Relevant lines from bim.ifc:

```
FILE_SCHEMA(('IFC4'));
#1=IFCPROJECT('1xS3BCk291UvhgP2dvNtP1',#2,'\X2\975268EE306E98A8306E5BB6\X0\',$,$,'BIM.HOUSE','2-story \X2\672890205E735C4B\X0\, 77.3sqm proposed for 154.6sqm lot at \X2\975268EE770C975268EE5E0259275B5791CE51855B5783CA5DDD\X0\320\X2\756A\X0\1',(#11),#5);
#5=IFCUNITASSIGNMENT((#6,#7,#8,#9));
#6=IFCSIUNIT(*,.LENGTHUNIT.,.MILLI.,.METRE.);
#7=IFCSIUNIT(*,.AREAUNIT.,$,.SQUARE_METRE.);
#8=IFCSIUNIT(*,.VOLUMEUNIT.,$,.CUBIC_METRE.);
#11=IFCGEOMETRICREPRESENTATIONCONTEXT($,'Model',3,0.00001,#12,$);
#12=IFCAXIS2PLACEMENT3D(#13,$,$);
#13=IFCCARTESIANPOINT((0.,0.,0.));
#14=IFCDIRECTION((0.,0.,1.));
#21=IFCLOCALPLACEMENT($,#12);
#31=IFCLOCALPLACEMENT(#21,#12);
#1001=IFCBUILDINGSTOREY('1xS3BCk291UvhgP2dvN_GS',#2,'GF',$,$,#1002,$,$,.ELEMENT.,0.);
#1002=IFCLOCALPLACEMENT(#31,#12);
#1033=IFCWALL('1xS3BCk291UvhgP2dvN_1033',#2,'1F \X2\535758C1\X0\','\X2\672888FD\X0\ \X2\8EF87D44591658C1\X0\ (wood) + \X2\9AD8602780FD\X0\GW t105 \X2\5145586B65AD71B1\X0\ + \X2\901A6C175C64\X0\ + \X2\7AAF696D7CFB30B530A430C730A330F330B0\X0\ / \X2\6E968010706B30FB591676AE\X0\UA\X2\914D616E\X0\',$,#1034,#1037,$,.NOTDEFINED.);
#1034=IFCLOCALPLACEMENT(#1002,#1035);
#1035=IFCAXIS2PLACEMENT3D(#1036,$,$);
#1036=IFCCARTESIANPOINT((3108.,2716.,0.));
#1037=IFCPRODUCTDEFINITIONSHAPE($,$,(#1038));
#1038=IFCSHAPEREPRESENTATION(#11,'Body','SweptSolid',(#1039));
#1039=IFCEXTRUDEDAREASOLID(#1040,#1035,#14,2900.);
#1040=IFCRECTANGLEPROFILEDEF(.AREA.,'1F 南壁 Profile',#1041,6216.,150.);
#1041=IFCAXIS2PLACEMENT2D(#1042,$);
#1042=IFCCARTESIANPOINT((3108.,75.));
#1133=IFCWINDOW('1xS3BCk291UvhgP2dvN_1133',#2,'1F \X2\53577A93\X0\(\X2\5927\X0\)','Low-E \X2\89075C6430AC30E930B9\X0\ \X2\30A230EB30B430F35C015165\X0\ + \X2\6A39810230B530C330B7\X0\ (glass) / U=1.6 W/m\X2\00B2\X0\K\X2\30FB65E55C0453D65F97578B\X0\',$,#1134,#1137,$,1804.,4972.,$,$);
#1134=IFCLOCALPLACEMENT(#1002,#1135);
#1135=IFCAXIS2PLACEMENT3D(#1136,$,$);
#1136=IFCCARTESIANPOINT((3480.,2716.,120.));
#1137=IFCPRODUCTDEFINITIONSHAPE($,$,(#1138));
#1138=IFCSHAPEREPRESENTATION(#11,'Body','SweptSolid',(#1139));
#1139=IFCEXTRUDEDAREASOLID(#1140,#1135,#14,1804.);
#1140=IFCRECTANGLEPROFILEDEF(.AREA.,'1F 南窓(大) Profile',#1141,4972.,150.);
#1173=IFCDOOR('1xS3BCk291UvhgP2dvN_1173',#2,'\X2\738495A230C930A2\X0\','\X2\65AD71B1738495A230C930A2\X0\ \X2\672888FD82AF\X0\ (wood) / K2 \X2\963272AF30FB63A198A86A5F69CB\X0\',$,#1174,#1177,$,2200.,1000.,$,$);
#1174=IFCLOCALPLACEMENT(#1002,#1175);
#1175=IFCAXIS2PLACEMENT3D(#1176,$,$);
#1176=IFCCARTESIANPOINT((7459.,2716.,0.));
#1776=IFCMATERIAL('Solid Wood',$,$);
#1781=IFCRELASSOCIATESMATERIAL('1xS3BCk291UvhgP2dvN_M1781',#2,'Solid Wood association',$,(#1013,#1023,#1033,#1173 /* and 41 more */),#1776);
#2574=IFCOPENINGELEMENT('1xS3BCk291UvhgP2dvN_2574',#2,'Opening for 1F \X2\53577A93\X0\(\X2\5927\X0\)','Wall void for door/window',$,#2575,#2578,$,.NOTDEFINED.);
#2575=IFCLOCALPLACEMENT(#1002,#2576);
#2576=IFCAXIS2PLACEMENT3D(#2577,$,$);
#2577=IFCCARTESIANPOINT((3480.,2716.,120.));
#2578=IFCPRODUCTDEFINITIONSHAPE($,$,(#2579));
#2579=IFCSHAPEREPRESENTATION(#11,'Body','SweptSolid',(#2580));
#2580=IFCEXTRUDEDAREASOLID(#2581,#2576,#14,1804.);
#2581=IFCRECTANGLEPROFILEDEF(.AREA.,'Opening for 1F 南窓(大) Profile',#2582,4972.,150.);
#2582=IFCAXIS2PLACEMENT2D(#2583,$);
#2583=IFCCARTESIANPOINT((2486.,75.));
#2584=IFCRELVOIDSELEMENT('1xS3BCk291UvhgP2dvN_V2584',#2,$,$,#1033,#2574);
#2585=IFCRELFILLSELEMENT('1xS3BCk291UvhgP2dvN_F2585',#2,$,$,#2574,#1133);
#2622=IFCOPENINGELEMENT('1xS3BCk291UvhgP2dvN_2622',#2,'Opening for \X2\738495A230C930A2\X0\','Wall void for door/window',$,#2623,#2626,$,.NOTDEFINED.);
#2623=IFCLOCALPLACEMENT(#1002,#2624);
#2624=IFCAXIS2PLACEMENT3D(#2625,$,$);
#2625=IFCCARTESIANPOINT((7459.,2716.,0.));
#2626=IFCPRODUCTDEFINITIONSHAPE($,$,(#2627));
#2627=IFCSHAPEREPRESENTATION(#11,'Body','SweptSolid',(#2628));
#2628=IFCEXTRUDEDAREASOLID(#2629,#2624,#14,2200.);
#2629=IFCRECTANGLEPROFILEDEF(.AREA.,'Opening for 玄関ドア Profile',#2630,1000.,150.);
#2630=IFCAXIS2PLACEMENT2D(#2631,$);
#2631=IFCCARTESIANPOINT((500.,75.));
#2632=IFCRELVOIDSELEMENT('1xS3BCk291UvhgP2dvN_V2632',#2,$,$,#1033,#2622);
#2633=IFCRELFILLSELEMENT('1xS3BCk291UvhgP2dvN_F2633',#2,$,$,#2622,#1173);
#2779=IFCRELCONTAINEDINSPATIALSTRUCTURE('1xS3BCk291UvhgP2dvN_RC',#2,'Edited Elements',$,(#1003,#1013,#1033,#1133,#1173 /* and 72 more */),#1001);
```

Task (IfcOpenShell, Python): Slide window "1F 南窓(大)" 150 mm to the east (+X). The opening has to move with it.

```python
import ifcopenshell
import ifcopenshell.api.geometry
import ifcopenshell.util.placement
import ifcopenshell.util.unit

model = ifcopenshell.open("bim.ifc")
unit_scale = ifcopenshell.util.unit.calculate_unit_scale(model)

window = model.by_id(1133)
opening = window.FillsVoids[0].RelatingOpeningElement
wall = opening.VoidsElements[0].RelatingBuildingElement

wall_matrix = ifcopenshell.util.placement.get_local_placement(wall.ObjectPlacement)
shift = wall_matrix[:3, 0] * 0.15 / unit_scale
before = ifcopenshell.util.placement.get_local_placement(window.ObjectPlacement)[:3, 3].copy()

# The window is not placed relative to its opening, so move both.
for product in (opening, window):
    matrix = ifcopenshell.util.placement.get_local_placement(product.ObjectPlacement)
    matrix[:3, 3] += shift
    ifcopenshell.api.geometry.edit_object_placement(model, product=product, matrix=matrix, is_si=False)

after = ifcopenshell.util.placement.get_local_placement(window.ObjectPlacement)[:3, 3]
print("window moved by", (after - before).round(3) + 0.0)

model.write("bim_edited.ifc")
```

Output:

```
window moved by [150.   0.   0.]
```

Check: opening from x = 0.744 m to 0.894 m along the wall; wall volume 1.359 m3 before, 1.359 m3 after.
